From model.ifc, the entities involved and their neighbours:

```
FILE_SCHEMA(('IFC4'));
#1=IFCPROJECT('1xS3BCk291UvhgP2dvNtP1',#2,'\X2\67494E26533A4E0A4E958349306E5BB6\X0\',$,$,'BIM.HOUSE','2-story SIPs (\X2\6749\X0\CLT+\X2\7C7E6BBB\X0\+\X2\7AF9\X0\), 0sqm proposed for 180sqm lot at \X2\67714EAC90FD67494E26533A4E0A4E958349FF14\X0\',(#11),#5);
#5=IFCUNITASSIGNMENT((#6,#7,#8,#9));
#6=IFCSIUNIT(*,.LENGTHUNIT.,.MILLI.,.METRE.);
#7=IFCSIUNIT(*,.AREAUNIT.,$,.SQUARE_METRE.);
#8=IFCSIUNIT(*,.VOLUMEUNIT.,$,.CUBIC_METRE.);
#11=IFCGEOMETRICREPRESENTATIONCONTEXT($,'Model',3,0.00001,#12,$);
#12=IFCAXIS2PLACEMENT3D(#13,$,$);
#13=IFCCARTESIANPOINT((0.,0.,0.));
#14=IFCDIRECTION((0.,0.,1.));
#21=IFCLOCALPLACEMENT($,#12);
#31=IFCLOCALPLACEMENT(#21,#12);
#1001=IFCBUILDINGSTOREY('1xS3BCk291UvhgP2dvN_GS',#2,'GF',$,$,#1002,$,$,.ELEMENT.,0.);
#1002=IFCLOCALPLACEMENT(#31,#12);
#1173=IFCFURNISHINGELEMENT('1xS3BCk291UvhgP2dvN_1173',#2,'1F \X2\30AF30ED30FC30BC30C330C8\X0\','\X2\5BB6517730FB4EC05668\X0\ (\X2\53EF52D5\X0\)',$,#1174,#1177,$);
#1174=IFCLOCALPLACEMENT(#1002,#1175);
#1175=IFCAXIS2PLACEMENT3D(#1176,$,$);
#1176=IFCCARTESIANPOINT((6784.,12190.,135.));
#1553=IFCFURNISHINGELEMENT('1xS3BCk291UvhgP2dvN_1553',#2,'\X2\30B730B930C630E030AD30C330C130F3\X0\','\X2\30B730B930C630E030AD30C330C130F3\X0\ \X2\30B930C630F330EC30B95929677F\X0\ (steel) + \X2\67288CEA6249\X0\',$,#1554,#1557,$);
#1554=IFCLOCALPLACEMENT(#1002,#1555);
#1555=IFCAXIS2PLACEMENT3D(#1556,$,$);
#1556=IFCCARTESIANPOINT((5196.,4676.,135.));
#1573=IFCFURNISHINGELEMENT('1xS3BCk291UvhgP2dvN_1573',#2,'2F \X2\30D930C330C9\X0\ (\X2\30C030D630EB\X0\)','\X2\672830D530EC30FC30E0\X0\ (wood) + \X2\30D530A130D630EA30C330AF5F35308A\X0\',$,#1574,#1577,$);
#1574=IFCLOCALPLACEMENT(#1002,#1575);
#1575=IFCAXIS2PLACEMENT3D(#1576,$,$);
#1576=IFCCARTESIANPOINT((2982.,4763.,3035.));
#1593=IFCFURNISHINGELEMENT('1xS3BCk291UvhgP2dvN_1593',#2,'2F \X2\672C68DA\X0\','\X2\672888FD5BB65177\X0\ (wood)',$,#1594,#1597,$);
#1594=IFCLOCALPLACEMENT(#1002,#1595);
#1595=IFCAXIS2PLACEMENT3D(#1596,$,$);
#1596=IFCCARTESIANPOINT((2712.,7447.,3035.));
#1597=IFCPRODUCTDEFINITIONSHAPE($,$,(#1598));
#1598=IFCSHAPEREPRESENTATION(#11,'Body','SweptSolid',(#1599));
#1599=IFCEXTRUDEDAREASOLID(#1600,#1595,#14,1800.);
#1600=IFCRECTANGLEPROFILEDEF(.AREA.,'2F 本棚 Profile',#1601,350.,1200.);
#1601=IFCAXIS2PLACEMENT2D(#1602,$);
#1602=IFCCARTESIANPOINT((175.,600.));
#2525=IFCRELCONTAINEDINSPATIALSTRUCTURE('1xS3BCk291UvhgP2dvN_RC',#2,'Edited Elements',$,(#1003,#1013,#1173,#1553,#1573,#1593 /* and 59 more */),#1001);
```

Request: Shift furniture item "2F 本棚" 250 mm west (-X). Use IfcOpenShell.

```python
import ifcopenshell
import ifcopenshell.api.geometry
import ifcopenshell.util.placement
import ifcopenshell.util.unit

model = ifcopenshell.open("model.ifc")
unit_scale = ifcopenshell.util.unit.calculate_unit_scale(model)

item = model.by_guid("1xS3BCk291UvhgP2dvN_1593")
matrix = ifcopenshell.util.placement.get_local_placement(item.ObjectPlacement)
matrix[0, 3] -= 0.25 / unit_scale
ifcopenshell.api.geometry.edit_object_placement(model, product=item, matrix=matrix, is_si=False)

print(ifcopenshell.util.placement.get_local_placement(item.ObjectPlacement).round(3) + 0.0)

model.write("model_edited.ifc")
```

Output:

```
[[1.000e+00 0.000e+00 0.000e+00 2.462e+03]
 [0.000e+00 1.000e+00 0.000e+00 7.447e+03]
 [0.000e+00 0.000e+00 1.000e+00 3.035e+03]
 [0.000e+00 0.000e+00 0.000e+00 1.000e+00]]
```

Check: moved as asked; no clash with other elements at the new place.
